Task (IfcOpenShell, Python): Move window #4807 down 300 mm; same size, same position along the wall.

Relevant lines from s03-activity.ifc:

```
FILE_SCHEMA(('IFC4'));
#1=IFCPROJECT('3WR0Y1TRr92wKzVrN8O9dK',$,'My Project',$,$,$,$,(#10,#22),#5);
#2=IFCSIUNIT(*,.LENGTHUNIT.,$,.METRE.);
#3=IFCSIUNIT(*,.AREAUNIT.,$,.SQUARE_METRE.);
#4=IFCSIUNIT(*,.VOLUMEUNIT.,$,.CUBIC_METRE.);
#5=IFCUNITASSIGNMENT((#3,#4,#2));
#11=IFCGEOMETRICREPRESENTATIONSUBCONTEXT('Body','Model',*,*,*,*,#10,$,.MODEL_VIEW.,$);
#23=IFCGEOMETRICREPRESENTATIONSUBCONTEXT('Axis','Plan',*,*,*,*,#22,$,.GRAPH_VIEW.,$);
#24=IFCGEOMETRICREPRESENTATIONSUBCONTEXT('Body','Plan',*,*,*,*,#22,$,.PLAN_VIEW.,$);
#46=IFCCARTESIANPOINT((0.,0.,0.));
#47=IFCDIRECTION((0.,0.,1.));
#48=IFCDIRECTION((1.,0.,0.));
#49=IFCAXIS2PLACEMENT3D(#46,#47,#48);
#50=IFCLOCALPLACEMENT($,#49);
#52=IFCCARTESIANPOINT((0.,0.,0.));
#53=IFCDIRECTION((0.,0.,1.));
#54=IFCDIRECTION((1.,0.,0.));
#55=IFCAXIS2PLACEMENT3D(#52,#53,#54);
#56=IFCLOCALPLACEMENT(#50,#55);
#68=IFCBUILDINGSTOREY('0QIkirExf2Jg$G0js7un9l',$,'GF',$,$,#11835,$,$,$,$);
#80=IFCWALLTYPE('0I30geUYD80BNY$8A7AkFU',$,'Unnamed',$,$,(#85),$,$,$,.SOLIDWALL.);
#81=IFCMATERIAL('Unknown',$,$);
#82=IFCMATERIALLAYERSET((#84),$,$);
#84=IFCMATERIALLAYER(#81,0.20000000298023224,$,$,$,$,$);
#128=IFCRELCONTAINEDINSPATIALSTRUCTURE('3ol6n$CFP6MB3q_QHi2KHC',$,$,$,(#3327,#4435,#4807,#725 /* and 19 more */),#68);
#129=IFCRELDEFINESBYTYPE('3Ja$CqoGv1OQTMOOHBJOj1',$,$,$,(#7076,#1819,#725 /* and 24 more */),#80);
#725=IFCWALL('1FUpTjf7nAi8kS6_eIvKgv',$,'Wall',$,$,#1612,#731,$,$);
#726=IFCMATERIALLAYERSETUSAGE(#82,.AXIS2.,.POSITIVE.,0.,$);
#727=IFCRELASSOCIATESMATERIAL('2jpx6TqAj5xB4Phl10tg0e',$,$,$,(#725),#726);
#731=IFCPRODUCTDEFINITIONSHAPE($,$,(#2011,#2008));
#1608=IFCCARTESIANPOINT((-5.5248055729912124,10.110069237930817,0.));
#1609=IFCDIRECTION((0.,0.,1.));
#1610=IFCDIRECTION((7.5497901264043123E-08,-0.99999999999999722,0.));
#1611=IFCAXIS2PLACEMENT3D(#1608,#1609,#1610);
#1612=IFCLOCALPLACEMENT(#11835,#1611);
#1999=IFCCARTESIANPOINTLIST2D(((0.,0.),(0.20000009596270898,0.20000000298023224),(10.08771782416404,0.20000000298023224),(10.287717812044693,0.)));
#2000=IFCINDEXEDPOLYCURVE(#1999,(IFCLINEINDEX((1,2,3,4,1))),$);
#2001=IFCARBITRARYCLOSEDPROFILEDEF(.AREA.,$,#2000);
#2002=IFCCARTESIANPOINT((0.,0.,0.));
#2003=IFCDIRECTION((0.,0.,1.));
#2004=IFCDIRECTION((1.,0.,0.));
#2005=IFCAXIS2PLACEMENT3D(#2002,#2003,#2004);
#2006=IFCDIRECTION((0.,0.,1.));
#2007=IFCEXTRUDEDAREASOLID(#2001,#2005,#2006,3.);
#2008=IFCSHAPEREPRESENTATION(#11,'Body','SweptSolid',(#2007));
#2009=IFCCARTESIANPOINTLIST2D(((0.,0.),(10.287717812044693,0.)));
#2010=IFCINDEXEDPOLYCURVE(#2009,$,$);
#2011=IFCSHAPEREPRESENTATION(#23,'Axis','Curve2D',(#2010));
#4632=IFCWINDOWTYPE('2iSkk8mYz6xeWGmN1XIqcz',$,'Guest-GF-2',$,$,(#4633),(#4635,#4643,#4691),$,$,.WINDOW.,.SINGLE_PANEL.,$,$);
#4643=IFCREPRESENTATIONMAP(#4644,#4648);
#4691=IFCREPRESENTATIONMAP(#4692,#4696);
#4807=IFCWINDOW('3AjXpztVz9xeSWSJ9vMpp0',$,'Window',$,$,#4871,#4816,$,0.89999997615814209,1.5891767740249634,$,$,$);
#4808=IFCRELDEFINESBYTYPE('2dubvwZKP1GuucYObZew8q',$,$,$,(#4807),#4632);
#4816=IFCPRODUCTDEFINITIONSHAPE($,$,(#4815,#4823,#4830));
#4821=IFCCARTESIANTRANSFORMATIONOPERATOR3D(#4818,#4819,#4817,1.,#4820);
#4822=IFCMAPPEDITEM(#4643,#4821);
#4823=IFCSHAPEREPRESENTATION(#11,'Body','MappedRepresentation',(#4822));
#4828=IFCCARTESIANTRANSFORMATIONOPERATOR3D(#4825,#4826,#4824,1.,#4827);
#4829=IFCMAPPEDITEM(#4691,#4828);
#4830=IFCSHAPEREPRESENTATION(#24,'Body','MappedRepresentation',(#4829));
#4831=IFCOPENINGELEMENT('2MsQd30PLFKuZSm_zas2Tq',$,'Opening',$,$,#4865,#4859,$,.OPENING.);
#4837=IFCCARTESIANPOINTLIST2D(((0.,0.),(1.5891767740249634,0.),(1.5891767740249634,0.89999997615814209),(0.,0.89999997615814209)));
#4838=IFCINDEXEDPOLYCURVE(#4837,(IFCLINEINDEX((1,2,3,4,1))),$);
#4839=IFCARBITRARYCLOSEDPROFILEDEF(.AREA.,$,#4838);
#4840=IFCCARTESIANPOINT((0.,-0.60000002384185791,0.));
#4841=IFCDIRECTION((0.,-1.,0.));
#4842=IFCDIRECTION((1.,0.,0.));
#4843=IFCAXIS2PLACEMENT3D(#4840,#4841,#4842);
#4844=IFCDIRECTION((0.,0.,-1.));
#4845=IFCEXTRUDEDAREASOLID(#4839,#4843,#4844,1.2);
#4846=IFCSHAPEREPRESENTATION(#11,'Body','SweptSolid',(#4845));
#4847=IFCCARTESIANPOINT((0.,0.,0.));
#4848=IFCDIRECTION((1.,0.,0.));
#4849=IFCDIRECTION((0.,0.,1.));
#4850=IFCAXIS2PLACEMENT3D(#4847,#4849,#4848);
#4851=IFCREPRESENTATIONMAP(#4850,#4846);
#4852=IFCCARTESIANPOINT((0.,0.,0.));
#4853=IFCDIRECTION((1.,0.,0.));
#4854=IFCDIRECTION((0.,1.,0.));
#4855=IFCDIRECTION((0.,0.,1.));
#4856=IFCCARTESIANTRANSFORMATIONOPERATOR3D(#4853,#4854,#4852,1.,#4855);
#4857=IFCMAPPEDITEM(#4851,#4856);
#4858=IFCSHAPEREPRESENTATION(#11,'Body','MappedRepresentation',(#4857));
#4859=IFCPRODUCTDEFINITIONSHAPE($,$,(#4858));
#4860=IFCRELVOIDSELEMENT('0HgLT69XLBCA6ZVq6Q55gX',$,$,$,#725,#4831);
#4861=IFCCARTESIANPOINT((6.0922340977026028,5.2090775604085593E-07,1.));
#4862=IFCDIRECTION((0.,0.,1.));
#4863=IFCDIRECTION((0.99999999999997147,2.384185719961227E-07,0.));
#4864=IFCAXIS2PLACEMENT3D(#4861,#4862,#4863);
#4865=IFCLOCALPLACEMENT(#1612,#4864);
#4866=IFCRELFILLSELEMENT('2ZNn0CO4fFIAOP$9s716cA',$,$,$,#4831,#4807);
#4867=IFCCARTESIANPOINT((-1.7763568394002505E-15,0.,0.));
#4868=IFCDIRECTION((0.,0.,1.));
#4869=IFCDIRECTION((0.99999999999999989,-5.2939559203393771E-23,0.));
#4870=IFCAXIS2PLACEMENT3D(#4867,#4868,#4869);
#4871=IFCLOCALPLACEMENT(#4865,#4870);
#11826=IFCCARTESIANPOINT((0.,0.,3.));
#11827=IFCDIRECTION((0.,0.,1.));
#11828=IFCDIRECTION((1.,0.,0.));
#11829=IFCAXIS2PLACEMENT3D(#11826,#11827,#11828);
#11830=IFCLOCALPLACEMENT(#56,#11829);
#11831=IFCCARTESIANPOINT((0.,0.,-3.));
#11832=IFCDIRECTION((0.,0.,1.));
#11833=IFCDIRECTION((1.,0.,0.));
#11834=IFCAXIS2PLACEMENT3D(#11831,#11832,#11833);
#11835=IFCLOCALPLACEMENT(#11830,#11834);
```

```python
import numpy as np
import ifcopenshell
import ifcopenshell.api.geometry
import ifcopenshell.util.placement
import ifcopenshell.util.unit

model = ifcopenshell.open("s03-activity.ifc")
unit_scale = ifcopenshell.util.unit.calculate_unit_scale(model)

window = model.by_guid("3AjXpztVz9xeSWSJ9vMpp0")
opening = window.FillsVoids[0].RelatingOpeningElement
dz = -0.3 / unit_scale

shift = np.array([0.0, 0.0, dz])
# The window is placed relative to its opening, so it follows when the opening moves.
matrix = ifcopenshell.util.placement.get_local_placement(opening.ObjectPlacement)
matrix[:3, 3] += shift
ifcopenshell.api.geometry.edit_object_placement(
    model, product=opening, matrix=matrix, is_si=False, should_transform_children=True
)

print(f"moved by {dz * unit_scale:+.3f} m")

model.write("s03-activity_v2.ifc")
```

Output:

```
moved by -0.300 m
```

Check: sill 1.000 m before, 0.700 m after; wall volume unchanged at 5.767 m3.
